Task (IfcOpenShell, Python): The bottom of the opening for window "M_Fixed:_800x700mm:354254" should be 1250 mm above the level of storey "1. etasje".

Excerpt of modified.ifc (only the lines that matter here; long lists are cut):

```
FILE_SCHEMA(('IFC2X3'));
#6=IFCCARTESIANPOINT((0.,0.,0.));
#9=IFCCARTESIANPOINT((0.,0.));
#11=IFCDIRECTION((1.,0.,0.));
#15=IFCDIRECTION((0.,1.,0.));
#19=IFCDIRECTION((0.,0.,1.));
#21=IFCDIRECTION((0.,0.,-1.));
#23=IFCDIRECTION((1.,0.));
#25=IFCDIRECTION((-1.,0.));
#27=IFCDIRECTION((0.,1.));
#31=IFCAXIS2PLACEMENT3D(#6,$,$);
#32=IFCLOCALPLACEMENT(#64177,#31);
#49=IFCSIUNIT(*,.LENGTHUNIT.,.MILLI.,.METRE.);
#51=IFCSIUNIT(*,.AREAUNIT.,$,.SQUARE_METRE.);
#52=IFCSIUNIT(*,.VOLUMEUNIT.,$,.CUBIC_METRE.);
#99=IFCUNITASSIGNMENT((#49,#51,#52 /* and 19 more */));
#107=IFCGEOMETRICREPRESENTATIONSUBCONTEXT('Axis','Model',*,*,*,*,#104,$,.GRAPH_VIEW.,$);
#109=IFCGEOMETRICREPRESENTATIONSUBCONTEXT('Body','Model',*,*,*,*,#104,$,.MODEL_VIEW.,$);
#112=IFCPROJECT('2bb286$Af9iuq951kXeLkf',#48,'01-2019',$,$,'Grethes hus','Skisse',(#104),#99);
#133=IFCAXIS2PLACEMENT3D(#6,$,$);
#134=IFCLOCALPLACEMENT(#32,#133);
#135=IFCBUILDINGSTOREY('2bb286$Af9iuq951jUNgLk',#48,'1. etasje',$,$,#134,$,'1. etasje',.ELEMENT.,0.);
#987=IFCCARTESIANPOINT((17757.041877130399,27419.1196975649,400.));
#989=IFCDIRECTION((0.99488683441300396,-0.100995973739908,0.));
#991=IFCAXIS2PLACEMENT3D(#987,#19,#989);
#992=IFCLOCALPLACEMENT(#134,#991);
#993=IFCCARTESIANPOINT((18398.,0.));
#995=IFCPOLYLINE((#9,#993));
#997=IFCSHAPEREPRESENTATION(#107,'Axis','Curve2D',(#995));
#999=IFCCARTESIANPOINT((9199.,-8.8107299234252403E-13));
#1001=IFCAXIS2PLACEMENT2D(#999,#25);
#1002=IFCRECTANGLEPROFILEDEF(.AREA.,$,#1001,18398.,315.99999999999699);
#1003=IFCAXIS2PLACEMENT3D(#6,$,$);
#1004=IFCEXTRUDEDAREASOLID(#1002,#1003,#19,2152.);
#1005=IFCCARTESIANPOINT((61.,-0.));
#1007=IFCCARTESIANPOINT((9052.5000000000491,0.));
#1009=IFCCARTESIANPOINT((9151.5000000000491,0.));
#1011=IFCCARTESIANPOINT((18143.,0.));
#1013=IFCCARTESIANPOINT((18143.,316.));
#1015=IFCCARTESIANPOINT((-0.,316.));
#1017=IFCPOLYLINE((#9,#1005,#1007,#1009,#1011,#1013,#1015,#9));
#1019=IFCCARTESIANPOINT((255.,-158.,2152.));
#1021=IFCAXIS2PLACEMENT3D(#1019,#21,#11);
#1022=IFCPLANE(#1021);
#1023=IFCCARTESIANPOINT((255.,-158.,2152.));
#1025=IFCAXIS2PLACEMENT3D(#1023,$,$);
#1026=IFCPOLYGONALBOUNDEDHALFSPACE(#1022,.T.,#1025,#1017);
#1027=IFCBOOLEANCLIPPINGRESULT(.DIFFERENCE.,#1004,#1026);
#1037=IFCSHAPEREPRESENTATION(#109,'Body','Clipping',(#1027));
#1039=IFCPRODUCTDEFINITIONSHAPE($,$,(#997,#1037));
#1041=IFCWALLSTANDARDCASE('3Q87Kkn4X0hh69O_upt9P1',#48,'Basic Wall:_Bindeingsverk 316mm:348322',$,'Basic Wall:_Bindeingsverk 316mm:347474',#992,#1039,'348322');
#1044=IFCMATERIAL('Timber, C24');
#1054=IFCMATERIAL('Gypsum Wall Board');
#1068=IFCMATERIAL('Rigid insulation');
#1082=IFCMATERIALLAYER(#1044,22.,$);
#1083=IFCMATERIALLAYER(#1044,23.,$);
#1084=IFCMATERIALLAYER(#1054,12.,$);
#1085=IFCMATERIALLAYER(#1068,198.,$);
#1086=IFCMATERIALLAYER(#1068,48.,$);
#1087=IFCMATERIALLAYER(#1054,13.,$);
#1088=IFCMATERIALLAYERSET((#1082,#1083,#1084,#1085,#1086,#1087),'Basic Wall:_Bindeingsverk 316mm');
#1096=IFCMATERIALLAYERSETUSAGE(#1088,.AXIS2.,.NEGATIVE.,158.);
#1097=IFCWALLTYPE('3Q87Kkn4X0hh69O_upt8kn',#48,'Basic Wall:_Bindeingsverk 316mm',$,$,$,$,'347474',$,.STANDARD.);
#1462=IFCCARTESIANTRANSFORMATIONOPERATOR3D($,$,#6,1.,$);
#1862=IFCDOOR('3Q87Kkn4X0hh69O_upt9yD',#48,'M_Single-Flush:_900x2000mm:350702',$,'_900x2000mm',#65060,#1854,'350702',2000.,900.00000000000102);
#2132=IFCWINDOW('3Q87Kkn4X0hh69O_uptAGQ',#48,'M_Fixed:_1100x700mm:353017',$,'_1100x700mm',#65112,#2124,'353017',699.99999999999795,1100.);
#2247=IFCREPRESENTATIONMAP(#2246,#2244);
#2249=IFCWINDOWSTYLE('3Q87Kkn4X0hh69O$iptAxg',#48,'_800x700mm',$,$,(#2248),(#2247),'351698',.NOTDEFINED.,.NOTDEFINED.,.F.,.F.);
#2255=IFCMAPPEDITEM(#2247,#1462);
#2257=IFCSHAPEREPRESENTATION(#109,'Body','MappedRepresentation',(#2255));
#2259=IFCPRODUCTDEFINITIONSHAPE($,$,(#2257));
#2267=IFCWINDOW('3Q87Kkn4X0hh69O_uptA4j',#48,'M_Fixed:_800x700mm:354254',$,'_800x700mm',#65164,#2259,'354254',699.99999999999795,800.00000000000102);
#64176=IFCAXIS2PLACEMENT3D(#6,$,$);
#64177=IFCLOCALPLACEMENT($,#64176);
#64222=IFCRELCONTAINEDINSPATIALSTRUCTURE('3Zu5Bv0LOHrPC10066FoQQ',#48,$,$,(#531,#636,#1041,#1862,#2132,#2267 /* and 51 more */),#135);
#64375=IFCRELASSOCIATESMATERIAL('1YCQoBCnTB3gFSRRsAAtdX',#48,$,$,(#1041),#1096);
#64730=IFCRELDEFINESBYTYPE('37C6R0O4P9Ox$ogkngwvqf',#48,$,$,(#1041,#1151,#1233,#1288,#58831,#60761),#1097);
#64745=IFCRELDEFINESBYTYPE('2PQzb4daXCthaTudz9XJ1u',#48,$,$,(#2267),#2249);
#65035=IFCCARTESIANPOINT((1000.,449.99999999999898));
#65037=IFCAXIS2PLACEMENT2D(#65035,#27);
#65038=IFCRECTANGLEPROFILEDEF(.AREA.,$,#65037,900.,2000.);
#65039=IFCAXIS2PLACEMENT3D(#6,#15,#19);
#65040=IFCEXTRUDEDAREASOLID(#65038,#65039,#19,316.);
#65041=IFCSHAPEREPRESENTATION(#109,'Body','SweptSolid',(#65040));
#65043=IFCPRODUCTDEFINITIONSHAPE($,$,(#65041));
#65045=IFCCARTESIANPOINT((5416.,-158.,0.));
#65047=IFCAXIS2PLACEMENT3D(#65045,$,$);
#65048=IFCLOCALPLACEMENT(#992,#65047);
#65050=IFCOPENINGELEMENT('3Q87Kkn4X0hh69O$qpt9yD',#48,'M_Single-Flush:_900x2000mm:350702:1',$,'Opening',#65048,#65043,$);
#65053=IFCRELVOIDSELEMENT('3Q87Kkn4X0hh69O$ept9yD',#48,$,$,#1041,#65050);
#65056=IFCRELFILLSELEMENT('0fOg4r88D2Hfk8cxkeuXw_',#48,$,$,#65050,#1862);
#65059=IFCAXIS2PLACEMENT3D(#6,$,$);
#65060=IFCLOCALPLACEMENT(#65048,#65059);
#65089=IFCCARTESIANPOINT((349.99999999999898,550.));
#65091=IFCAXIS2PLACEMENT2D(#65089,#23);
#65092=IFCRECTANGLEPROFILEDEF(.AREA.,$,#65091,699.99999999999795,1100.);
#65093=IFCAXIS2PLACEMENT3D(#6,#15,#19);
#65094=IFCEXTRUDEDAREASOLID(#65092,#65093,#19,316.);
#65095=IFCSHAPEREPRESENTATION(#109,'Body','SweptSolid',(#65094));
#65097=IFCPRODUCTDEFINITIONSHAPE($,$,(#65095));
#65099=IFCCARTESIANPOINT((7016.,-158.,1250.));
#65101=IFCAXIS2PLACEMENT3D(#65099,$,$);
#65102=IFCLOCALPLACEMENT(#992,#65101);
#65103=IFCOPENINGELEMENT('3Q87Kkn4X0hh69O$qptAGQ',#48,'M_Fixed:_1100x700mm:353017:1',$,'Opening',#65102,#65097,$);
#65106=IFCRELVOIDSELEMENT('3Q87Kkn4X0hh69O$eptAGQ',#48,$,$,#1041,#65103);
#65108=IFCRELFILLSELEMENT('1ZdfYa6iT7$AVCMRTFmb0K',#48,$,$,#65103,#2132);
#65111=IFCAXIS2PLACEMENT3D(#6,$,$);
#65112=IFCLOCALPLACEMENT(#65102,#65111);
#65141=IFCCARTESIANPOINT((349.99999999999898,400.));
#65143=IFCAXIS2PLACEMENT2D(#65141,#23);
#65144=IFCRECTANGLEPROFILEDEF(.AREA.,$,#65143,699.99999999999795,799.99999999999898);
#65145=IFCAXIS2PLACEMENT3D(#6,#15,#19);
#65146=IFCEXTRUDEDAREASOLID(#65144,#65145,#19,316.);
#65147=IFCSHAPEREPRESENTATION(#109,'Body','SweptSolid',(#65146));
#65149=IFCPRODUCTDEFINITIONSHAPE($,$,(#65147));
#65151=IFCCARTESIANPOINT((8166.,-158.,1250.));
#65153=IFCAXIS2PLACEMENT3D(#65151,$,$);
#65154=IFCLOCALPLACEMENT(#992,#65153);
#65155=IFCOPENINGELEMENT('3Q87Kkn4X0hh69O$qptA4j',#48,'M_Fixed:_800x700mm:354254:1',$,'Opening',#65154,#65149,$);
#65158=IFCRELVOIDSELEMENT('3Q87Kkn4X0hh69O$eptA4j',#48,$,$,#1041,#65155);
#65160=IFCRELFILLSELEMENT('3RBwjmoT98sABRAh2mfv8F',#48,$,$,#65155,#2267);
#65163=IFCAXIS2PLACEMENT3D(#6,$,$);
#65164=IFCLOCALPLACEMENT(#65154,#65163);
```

```python
import numpy as np
import ifcopenshell
import ifcopenshell.api.geometry
import ifcopenshell.geom
import ifcopenshell.util.element
import ifcopenshell.util.placement
import ifcopenshell.util.shape
import ifcopenshell.util.unit

model = ifcopenshell.open("modified.ifc")
unit_scale = ifcopenshell.util.unit.calculate_unit_scale(model)

window = model.by_guid("3Q87Kkn4X0hh69O_uptA4j")
opening = window.FillsVoids[0].RelatingOpeningElement
storey = ifcopenshell.util.element.get_container(window, ifc_class="IfcBuildingStorey")
level = ifcopenshell.util.placement.get_local_placement(storey.ObjectPlacement)[2, 3]

# The opening's origin need not be at the sill, so measure its lowest point.
shape = ifcopenshell.geom.create_shape(ifcopenshell.geom.settings(), opening)
bottom = ifcopenshell.util.shape.get_shape_bottom_elevation(shape, shape.geometry) / unit_scale
dz = level + 1.25 / unit_scale - bottom

shift = np.array([0.0, 0.0, dz])
# The window is placed relative to its opening, so it follows when the opening moves.
matrix = ifcopenshell.util.placement.get_local_placement(opening.ObjectPlacement)
matrix[:3, 3] += shift
ifcopenshell.api.geometry.edit_object_placement(
    model, product=opening, matrix=matrix, is_si=False, should_transform_children=True
)

print(f"moved by {dz * unit_scale:+.3f} m")

model.write("modified_rev.ifc")
```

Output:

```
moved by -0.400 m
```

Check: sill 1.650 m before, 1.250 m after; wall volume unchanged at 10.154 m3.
